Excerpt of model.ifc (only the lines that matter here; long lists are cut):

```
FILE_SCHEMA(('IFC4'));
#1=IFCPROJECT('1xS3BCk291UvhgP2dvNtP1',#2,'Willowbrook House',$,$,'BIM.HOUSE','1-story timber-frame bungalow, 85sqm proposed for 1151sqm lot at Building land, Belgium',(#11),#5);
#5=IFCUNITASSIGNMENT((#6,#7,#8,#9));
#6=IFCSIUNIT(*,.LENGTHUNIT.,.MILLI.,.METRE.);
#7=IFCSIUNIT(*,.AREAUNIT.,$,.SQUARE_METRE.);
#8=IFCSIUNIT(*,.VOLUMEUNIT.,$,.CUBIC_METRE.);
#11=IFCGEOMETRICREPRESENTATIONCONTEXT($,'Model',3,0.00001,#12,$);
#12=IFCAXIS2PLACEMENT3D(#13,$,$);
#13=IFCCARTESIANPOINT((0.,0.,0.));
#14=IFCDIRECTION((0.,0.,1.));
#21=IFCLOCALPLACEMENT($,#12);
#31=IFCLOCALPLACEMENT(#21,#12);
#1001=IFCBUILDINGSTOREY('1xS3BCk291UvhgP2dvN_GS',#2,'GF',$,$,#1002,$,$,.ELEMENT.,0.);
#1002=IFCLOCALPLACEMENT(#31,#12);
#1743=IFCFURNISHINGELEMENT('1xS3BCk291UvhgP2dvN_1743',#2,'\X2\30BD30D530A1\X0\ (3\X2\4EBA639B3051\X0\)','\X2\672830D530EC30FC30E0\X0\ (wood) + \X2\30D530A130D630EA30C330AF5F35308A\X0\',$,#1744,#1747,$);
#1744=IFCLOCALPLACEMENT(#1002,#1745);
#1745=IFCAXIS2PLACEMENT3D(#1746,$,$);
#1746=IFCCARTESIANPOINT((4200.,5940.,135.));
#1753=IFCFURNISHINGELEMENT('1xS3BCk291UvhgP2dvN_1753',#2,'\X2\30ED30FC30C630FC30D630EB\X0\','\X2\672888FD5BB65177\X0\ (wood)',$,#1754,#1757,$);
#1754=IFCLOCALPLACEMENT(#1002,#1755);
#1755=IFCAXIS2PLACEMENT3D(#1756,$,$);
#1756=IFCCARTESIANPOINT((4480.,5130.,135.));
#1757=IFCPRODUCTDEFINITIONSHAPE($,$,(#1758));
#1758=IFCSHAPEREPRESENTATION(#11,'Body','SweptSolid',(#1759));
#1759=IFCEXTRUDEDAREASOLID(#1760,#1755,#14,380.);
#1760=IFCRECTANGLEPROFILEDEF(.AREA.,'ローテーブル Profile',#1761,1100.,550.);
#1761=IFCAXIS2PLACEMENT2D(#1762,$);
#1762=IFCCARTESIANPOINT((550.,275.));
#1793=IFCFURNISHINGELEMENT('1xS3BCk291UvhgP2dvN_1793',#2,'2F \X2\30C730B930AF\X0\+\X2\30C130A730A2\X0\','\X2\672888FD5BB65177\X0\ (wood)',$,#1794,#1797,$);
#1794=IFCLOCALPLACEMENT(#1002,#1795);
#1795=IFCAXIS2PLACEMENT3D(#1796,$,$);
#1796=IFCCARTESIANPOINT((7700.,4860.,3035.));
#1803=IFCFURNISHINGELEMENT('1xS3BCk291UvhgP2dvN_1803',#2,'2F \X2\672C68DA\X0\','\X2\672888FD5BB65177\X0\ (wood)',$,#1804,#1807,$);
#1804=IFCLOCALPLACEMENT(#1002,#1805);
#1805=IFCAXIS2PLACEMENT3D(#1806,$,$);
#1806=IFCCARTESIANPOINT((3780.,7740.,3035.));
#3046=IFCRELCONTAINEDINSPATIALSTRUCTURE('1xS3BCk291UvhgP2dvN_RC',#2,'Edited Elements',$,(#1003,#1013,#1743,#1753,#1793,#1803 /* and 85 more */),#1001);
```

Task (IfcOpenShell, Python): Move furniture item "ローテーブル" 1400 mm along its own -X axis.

```python
import ifcopenshell
import ifcopenshell.api.geometry
import ifcopenshell.util.placement

model = ifcopenshell.open("model.ifc")

item = model.by_guid("1xS3BCk291UvhgP2dvN_1753")
matrix = ifcopenshell.util.placement.get_local_placement(item.ObjectPlacement)
matrix[:3, 3] -= matrix[:3, 0] * 1400.0
ifcopenshell.api.geometry.edit_object_placement(model, product=item, matrix=matrix, is_si=False)

print(ifcopenshell.util.placement.get_local_placement(item.ObjectPlacement).round(3) + 0.0)

model.write("model_updated.ifc")
```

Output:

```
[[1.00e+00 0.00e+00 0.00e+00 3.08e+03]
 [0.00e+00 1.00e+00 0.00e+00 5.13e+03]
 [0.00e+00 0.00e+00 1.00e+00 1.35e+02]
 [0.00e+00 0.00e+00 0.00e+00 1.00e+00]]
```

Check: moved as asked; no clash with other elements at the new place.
